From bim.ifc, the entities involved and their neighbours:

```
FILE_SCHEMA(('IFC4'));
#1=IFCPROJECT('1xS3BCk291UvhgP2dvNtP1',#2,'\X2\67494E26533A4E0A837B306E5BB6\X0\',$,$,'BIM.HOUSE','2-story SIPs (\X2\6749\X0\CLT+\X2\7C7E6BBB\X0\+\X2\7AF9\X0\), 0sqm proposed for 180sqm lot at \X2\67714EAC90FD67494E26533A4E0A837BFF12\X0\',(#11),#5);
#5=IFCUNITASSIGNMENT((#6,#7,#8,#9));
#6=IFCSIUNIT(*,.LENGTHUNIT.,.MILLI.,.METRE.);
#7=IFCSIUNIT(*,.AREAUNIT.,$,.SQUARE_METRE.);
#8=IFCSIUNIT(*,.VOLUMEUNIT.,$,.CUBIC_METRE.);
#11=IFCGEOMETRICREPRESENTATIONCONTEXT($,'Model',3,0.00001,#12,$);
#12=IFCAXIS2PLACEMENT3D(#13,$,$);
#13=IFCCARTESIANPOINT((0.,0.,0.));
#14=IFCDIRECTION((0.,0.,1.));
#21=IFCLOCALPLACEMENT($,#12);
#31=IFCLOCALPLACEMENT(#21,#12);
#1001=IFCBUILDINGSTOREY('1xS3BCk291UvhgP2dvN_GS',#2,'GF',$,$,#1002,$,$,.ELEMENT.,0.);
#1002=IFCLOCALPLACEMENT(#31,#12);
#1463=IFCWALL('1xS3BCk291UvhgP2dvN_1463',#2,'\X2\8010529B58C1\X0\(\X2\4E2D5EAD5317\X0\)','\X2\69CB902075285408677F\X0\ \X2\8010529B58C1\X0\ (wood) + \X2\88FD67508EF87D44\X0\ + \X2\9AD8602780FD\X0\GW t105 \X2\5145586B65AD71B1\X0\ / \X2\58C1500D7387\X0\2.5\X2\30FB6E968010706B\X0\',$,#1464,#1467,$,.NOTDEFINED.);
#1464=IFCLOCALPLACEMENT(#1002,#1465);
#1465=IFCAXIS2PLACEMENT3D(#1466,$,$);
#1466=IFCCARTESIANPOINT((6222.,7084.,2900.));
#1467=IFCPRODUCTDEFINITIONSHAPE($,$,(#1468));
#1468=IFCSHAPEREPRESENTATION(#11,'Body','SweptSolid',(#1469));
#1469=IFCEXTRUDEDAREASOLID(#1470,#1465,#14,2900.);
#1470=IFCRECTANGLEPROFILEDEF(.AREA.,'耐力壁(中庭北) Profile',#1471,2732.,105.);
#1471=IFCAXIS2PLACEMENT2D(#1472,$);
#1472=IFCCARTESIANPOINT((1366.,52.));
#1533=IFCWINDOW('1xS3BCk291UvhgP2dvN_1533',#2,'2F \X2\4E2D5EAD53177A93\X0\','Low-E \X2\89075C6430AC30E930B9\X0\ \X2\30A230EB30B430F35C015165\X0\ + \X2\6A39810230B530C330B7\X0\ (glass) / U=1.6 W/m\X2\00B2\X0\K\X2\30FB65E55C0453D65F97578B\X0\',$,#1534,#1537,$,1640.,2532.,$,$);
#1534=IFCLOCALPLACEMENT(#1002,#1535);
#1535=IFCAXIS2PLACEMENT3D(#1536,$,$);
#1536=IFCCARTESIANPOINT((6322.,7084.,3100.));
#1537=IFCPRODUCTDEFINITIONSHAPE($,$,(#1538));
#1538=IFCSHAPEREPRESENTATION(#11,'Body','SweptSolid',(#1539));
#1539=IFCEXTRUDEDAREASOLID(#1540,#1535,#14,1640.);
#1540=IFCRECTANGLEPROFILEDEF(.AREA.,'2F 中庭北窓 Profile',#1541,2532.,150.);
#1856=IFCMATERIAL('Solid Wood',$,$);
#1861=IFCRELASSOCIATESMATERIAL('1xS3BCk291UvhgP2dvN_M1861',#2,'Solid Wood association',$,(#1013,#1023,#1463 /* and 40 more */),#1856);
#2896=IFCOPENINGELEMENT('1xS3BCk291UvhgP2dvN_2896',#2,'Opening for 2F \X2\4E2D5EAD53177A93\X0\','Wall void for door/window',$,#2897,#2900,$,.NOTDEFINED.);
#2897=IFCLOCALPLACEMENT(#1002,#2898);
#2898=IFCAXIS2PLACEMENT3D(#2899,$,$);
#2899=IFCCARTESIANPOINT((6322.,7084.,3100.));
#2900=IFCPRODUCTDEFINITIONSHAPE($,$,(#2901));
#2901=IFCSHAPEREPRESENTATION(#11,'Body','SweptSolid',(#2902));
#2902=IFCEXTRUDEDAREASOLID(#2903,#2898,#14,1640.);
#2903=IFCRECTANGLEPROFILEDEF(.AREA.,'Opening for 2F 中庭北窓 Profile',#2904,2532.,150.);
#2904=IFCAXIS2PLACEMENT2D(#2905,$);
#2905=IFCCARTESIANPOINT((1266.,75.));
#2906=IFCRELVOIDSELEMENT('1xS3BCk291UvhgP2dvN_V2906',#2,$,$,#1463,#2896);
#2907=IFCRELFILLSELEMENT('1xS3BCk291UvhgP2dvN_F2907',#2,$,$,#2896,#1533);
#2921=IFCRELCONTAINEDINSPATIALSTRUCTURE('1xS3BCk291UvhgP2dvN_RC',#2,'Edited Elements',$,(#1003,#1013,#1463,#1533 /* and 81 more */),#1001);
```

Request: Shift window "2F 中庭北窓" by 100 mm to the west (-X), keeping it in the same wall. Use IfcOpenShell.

```python
import ifcopenshell
import ifcopenshell.api.geometry
import ifcopenshell.util.placement

model = ifcopenshell.open("bim.ifc")

window = model.by_guid("1xS3BCk291UvhgP2dvN_1533")
opening = window.FillsVoids[0].RelatingOpeningElement
wall = opening.VoidsElements[0].RelatingBuildingElement

wall_matrix = ifcopenshell.util.placement.get_local_placement(wall.ObjectPlacement)
shift = wall_matrix[:3, 0] * -100.0
before = ifcopenshell.util.placement.get_local_placement(window.ObjectPlacement)[:3, 3].copy()

# The window is not placed relative to its opening, so move both.
for product in (opening, window):
    matrix = ifcopenshell.util.placement.get_local_placement(product.ObjectPlacement)
    matrix[:3, 3] += shift
    ifcopenshell.api.geometry.edit_object_placement(model, product=product, matrix=matrix, is_si=False)

after = ifcopenshell.util.placement.get_local_placement(window.ObjectPlacement)[:3, 3]
print("window moved by", (after - before).round(3) + 0.0)

model.write("bim_edited.ifc")
```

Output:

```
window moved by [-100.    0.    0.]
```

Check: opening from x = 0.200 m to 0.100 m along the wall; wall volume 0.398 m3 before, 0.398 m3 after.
